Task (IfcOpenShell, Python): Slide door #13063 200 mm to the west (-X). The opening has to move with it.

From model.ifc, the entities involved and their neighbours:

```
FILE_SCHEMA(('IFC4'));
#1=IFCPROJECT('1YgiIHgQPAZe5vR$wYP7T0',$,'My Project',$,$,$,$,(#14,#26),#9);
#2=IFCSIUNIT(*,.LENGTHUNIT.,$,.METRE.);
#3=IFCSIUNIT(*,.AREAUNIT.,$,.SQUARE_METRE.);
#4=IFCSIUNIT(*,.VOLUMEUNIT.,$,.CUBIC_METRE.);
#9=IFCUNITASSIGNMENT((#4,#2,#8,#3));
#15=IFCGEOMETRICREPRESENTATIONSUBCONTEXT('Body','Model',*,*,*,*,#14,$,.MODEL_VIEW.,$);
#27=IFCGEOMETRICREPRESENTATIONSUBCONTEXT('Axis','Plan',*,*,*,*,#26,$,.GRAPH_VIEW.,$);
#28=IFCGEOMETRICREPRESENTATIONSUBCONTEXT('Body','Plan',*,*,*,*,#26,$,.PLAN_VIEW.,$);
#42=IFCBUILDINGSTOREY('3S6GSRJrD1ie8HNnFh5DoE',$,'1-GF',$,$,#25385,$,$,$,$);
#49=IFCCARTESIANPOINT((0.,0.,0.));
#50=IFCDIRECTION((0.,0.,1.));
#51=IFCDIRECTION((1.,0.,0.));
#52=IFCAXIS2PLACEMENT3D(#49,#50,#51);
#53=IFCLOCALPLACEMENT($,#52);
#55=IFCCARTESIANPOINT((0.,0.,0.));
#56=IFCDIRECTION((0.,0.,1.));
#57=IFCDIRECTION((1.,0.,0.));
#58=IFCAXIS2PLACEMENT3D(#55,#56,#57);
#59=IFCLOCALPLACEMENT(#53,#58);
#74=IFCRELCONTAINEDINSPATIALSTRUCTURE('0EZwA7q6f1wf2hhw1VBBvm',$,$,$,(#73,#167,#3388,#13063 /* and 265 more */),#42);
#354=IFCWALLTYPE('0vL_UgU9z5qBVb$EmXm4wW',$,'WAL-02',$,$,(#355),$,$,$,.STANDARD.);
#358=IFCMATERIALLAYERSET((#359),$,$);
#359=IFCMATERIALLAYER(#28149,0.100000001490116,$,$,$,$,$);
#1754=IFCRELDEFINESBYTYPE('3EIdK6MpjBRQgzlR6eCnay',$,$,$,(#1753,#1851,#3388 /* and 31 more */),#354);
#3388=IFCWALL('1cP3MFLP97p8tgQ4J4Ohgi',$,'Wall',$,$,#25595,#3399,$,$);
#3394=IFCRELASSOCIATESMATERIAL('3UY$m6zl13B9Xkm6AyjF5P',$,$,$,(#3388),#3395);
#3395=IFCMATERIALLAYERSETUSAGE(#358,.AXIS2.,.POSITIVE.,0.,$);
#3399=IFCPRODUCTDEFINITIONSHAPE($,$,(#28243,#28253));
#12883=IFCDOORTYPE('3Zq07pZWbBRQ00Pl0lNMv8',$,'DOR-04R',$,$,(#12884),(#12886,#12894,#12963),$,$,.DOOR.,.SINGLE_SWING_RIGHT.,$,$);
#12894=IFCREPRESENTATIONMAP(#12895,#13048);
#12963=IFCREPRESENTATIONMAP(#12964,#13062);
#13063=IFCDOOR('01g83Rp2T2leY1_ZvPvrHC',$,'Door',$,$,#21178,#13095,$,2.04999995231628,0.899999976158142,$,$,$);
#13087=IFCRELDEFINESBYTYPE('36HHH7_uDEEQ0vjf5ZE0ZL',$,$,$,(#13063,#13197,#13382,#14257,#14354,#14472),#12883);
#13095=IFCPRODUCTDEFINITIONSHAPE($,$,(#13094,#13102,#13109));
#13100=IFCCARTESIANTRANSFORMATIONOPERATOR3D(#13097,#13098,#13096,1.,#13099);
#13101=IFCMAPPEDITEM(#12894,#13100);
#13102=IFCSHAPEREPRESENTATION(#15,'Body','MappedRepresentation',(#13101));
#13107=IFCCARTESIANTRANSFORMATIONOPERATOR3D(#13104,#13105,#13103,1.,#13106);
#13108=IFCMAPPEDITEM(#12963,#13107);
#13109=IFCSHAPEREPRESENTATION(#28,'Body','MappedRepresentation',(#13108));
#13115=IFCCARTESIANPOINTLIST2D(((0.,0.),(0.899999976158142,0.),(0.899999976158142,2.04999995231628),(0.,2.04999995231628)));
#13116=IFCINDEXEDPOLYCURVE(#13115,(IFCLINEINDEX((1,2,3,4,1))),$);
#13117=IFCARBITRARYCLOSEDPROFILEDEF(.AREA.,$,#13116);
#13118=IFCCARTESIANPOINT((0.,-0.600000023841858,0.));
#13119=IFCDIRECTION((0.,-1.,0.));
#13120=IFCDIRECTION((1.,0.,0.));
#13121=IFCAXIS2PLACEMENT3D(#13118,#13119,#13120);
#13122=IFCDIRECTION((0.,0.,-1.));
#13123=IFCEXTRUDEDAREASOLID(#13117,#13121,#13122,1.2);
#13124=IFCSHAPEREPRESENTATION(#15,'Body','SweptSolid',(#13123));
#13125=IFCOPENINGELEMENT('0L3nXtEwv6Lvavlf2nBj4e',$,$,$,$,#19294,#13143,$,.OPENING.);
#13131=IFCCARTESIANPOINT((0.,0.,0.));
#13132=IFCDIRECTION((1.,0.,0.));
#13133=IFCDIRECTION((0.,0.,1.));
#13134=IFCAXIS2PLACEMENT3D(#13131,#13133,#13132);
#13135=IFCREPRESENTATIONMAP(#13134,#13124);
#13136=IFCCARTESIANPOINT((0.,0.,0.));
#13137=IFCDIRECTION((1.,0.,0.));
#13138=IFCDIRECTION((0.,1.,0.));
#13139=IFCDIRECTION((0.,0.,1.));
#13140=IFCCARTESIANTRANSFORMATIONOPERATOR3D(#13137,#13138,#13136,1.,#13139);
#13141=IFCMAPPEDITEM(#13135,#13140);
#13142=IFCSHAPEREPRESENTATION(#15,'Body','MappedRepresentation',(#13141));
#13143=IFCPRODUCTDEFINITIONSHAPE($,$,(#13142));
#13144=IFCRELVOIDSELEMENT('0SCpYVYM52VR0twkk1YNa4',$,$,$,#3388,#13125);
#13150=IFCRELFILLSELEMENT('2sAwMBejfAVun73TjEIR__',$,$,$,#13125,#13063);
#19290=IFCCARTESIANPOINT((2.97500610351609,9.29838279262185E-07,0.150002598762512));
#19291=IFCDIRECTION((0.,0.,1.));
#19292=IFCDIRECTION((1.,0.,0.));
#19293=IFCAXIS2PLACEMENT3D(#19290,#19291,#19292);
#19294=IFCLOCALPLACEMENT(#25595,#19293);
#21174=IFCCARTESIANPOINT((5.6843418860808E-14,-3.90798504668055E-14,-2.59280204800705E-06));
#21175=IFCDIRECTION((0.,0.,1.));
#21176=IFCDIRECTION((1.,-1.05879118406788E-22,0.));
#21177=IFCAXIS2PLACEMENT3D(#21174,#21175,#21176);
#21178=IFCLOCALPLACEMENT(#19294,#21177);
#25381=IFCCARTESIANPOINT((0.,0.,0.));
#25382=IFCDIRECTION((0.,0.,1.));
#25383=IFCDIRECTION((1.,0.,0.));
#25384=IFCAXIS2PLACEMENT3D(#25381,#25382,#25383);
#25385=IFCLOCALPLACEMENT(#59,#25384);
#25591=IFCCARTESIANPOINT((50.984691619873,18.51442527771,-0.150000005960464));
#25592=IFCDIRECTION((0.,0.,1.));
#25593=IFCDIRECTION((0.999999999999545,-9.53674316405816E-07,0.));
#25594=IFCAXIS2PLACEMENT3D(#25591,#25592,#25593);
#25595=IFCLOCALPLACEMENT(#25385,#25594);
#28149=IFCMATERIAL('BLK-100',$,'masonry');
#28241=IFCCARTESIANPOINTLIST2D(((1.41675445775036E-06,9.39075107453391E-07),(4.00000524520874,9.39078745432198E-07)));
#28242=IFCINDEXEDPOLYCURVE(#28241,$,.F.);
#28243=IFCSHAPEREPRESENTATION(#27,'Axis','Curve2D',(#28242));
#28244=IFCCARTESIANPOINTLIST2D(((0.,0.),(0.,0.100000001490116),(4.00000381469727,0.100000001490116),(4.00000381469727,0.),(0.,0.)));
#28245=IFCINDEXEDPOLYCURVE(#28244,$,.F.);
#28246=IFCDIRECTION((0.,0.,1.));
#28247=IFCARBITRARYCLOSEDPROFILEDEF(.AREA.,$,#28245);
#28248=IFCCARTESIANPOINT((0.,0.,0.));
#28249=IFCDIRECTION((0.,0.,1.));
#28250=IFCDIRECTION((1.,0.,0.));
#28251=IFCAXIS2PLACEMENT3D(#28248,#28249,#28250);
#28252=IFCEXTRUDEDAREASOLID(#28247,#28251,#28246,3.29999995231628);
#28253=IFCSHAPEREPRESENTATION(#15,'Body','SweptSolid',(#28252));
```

```python
import ifcopenshell
import ifcopenshell.api.geometry
import ifcopenshell.util.placement

model = ifcopenshell.open("model.ifc")

door = model.by_id(13063)
opening = door.FillsVoids[0].RelatingOpeningElement
wall = opening.VoidsElements[0].RelatingBuildingElement

wall_matrix = ifcopenshell.util.placement.get_local_placement(wall.ObjectPlacement)
shift = wall_matrix[:3, 0] * -0.2
before = ifcopenshell.util.placement.get_local_placement(door.ObjectPlacement)[:3, 3].copy()

# The door is placed relative to its opening, so it follows when the opening moves.
matrix = ifcopenshell.util.placement.get_local_placement(opening.ObjectPlacement)
matrix[:3, 3] += shift
ifcopenshell.api.geometry.edit_object_placement(
    model, product=opening, matrix=matrix, is_si=False, should_transform_children=True
)

after = ifcopenshell.util.placement.get_local_placement(door.ObjectPlacement)[:3, 3]
print("door moved by", (after - before).round(3) + 0.0)

model.write("model_rev.ifc")
```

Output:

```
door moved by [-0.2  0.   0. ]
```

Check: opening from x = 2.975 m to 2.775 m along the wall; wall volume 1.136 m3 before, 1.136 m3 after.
